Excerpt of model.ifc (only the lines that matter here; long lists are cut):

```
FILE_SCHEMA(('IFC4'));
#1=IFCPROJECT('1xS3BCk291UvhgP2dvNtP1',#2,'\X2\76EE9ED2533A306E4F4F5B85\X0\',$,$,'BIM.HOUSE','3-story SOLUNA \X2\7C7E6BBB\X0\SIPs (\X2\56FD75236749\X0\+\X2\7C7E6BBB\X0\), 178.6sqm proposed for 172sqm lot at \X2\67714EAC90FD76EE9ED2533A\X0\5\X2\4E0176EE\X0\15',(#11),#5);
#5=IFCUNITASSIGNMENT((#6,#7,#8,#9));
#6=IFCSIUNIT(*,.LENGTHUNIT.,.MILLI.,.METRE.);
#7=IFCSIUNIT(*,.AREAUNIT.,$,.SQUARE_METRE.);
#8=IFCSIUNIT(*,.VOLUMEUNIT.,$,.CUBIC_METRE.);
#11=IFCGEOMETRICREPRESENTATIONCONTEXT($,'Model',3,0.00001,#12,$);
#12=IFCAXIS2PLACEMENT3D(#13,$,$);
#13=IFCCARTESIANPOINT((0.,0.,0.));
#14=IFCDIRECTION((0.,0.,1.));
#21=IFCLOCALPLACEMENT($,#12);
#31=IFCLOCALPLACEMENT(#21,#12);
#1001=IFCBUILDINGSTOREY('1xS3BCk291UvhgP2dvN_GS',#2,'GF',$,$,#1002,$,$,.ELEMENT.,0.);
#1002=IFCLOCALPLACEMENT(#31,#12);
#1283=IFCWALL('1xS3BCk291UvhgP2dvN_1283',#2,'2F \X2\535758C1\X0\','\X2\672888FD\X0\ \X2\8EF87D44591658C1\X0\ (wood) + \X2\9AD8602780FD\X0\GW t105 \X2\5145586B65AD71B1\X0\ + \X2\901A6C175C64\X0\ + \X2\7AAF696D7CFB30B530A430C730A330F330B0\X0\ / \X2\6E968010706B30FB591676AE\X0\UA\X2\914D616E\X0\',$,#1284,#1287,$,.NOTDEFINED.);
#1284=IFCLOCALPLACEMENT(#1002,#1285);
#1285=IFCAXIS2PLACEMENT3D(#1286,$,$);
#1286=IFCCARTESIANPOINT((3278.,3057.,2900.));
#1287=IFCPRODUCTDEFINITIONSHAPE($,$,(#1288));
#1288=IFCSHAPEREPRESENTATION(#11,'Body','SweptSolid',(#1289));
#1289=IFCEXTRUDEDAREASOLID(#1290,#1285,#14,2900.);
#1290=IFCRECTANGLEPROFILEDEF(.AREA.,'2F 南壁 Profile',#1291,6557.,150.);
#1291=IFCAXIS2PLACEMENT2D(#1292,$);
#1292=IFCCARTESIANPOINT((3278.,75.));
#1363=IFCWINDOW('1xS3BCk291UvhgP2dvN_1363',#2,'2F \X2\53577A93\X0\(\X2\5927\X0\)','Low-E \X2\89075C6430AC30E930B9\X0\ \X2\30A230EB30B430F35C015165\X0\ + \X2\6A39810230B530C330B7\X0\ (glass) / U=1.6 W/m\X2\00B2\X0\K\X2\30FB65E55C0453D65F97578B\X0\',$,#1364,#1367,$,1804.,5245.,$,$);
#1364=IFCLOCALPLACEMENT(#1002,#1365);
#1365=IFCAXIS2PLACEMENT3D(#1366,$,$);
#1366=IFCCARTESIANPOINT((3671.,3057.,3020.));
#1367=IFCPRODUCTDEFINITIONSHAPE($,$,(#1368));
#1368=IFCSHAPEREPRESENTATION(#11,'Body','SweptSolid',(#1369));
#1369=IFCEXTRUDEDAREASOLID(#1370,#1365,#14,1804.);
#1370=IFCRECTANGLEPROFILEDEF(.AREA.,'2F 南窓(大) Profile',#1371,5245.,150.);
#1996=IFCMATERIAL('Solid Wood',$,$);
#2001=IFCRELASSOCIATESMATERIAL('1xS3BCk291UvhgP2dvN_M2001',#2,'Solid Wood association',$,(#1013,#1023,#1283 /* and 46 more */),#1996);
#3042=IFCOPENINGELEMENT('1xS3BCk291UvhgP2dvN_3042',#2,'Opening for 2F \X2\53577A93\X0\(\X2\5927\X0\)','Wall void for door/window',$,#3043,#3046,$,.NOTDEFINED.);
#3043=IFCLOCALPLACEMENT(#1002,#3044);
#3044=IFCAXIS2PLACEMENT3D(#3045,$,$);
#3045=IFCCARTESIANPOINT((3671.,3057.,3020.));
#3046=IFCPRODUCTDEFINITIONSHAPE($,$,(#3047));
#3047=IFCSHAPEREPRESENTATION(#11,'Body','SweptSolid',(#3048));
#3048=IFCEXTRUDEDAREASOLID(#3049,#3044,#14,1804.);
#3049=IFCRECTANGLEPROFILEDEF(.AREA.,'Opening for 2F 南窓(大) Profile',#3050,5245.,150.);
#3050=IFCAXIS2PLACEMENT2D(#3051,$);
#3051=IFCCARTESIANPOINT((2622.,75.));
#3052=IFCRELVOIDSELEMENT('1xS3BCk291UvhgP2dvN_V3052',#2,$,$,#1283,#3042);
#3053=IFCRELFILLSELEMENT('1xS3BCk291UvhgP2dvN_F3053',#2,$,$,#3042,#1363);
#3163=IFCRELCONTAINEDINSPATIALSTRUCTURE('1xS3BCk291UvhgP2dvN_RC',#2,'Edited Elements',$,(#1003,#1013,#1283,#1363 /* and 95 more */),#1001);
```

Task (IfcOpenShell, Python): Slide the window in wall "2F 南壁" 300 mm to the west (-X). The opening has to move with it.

```python
import ifcopenshell
import ifcopenshell.api.geometry
import ifcopenshell.util.placement
import ifcopenshell.util.unit

model = ifcopenshell.open("model.ifc")
unit_scale = ifcopenshell.util.unit.calculate_unit_scale(model)

window = model.by_guid("1xS3BCk291UvhgP2dvN_1363")
opening = window.FillsVoids[0].RelatingOpeningElement
wall = opening.VoidsElements[0].RelatingBuildingElement

wall_matrix = ifcopenshell.util.placement.get_local_placement(wall.ObjectPlacement)
shift = wall_matrix[:3, 0] * -0.3 / unit_scale
before = ifcopenshell.util.placement.get_local_placement(window.ObjectPlacement)[:3, 3].copy()

# The window is not placed relative to its opening, so move both.
for product in (opening, window):
    matrix = ifcopenshell.util.placement.get_local_placement(product.ObjectPlacement)
    matrix[:3, 3] += shift
    ifcopenshell.api.geometry.edit_object_placement(model, product=product, matrix=matrix, is_si=False)

after = ifcopenshell.util.placement.get_local_placement(window.ObjectPlacement)[:3, 3]
print("window moved by", (after - before).round(3) + 0.0)

model.write("model_updated.ifc")
```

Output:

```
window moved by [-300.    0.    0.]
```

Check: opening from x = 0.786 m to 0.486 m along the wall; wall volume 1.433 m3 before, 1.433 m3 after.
